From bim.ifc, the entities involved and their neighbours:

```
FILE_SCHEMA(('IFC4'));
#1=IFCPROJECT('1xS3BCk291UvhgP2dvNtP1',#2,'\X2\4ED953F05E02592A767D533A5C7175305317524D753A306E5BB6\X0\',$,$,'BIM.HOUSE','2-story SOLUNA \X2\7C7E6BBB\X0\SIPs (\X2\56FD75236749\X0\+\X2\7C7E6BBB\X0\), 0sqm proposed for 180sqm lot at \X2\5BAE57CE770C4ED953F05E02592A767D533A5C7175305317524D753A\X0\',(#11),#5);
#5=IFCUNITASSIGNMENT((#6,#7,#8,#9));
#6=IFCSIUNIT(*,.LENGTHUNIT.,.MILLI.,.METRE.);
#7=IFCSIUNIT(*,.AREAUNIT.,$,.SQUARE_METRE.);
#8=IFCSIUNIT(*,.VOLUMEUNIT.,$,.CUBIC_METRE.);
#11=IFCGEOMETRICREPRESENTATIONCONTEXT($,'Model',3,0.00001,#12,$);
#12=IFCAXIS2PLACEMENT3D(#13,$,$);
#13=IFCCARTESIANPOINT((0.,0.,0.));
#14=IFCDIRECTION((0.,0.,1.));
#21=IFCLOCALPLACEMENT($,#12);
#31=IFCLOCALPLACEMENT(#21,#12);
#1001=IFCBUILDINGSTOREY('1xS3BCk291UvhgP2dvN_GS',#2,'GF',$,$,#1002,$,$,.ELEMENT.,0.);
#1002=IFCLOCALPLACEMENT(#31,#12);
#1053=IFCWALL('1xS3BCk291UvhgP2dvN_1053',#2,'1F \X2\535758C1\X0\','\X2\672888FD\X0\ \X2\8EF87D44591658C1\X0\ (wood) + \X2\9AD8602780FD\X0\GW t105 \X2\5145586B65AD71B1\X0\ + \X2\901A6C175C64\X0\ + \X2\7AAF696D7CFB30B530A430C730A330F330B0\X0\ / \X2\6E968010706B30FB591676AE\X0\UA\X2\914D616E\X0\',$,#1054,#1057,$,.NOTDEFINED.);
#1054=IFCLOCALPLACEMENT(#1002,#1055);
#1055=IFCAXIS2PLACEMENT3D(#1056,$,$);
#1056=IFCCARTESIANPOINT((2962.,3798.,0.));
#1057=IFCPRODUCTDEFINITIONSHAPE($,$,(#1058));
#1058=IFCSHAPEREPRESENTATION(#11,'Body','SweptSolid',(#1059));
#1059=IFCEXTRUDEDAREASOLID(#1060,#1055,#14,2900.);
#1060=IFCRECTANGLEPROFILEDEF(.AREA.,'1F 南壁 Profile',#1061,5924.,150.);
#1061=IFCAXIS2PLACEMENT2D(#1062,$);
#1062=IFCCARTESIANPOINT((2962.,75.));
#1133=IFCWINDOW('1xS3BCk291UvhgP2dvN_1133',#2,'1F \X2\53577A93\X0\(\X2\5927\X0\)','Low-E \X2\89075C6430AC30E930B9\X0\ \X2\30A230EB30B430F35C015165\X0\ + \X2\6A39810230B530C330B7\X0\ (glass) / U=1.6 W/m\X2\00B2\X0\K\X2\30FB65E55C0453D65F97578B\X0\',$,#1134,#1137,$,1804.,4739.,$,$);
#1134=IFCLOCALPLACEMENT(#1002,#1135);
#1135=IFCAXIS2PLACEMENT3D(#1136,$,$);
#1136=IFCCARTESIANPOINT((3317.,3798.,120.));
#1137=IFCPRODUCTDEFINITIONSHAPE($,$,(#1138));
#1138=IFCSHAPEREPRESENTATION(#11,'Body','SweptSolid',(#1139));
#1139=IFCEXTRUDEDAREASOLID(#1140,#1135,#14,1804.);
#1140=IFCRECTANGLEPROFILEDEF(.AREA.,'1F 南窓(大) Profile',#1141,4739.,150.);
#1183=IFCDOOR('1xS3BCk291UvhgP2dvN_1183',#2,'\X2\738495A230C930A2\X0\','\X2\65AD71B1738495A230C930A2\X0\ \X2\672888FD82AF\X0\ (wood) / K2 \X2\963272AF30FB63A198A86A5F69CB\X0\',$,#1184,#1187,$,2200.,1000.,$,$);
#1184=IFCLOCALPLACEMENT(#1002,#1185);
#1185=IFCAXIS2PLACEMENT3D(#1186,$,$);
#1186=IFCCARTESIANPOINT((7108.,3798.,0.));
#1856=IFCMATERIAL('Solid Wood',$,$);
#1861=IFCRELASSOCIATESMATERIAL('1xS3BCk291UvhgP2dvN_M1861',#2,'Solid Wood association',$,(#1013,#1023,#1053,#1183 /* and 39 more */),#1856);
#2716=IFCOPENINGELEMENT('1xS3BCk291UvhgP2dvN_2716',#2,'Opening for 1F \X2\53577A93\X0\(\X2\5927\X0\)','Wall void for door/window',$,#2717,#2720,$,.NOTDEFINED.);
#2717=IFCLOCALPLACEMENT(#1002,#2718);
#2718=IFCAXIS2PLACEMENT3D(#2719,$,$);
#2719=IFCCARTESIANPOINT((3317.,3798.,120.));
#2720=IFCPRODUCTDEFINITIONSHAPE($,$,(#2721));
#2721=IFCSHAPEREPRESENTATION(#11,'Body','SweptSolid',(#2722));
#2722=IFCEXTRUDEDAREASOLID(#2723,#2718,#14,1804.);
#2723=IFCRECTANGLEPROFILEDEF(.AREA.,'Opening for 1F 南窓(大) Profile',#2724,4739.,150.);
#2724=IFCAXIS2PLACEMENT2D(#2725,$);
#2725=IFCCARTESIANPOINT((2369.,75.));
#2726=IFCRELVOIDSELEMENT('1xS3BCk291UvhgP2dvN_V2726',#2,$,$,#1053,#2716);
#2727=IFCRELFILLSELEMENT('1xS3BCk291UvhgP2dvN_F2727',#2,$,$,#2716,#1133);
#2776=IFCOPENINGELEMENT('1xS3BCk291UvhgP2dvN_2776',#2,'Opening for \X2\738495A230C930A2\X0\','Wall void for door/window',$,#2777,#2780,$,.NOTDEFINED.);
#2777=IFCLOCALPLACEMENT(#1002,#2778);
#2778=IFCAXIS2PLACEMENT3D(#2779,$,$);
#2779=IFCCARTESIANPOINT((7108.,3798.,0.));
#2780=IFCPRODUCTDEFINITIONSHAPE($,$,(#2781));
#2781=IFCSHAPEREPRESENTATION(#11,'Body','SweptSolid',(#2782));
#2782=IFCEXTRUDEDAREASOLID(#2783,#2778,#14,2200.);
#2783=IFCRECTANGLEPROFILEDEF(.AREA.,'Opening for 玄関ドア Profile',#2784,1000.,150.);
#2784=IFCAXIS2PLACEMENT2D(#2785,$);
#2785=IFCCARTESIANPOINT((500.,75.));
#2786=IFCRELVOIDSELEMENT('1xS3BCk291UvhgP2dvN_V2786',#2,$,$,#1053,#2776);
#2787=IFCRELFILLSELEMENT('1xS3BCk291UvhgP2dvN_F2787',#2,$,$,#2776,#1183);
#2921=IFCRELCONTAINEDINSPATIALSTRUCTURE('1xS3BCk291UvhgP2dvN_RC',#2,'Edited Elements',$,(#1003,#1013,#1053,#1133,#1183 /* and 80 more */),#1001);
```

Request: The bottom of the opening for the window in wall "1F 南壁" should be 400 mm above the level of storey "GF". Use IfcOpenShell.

```python
import numpy as np
import ifcopenshell
import ifcopenshell.api.geometry
import ifcopenshell.geom
import ifcopenshell.util.element
import ifcopenshell.util.placement
import ifcopenshell.util.shape
import ifcopenshell.util.unit

model = ifcopenshell.open("bim.ifc")
unit_scale = ifcopenshell.util.unit.calculate_unit_scale(model)

window = model.by_guid("1xS3BCk291UvhgP2dvN_1133")
opening = window.FillsVoids[0].RelatingOpeningElement
storey = ifcopenshell.util.element.get_container(window, ifc_class="IfcBuildingStorey")
level = ifcopenshell.util.placement.get_local_placement(storey.ObjectPlacement)[2, 3]

# The opening's origin need not be at the sill, so measure its lowest point.
shape = ifcopenshell.geom.create_shape(ifcopenshell.geom.settings(), opening)
bottom = ifcopenshell.util.shape.get_shape_bottom_elevation(shape, shape.geometry) / unit_scale
dz = level + 0.4 / unit_scale - bottom

shift = np.array([0.0, 0.0, dz])
# The window is not placed relative to its opening, so move both.
for product in (opening, window):
    matrix = ifcopenshell.util.placement.get_local_placement(product.ObjectPlacement)
    matrix[:3, 3] += shift
    ifcopenshell.api.geometry.edit_object_placement(model, product=product, matrix=matrix, is_si=False)

print(f"moved by {dz * unit_scale:+.3f} m")

model.write("bim_v2.ifc")
```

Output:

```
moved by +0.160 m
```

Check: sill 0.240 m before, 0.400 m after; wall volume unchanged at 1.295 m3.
